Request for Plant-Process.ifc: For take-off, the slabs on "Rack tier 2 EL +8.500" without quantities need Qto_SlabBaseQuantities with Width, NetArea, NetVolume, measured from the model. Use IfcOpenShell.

First a look at what the model holds.

```python
import ifcopenshell
import ifcopenshell.util.element
import ifcopenshell.util.unit

model = ifcopenshell.open("Plant-Process.ifc")
print(model.schema)
for unit_type in ("LENGTHUNIT", "AREAUNIT", "VOLUMEUNIT"):
    print(unit_type, ifcopenshell.util.unit.calculate_unit_scale(model, unit_type))
storey = next(s for s in model.by_type("IfcBuildingStorey") if s.Name == "Rack tier 2 EL +8.500")
slabs = [e for e in ifcopenshell.util.element.get_decomposition(storey) if e.is_a("IfcSlab")]
for e in sorted(slabs, key=lambda e: e.id()):
    print(e.id(), e.is_a(), e.Name, list(ifcopenshell.util.element.get_psets(e, qtos_only=True)), sep=" | ")
```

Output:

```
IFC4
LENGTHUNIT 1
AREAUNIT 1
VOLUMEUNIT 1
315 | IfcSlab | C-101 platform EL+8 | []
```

```python
import ifcopenshell
import ifcopenshell.api.pset
import ifcopenshell.geom
import ifcopenshell.util.element
import ifcopenshell.util.shape
import ifcopenshell.util.unit

model = ifcopenshell.open("Plant-Process.ifc")
unit_scale = ifcopenshell.util.unit.calculate_unit_scale(model)
area_scale = ifcopenshell.util.unit.calculate_unit_scale(model, "AREAUNIT")
volume_scale = ifcopenshell.util.unit.calculate_unit_scale(model, "VOLUMEUNIT")
settings = ifcopenshell.geom.settings()

storey = next(s for s in model.by_type("IfcBuildingStorey") if s.Name == "Rack tier 2 EL +8.500")
slabs = [e for e in ifcopenshell.util.element.get_decomposition(storey) if e.is_a("IfcSlab")]

for e in sorted(slabs, key=lambda e: e.id()):
    if ifcopenshell.util.element.get_psets(e, qtos_only=True, should_inherit=False):
        continue
    # Geometry comes back in metres, in the element's own axes.
    shape = ifcopenshell.geom.create_shape(settings, e)
    values = {
        "Width": ifcopenshell.util.shape.get_z(shape.geometry) / unit_scale,
        "NetArea": ifcopenshell.util.shape.get_footprint_area(shape.geometry) / area_scale,
        "NetVolume": ifcopenshell.util.shape.get_volume(shape.geometry) / volume_scale,
    }
    qto = ifcopenshell.api.pset.add_qto(model, product=e, name="Qto_SlabBaseQuantities")
    ifcopenshell.api.pset.edit_qto(model, qto=qto, properties=values)
    print(e.id(), {k: round(v, 3) for k, v in values.items()})

model.write("Plant-Process_updated.ifc")
```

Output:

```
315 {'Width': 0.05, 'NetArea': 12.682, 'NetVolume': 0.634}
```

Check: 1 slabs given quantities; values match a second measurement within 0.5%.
